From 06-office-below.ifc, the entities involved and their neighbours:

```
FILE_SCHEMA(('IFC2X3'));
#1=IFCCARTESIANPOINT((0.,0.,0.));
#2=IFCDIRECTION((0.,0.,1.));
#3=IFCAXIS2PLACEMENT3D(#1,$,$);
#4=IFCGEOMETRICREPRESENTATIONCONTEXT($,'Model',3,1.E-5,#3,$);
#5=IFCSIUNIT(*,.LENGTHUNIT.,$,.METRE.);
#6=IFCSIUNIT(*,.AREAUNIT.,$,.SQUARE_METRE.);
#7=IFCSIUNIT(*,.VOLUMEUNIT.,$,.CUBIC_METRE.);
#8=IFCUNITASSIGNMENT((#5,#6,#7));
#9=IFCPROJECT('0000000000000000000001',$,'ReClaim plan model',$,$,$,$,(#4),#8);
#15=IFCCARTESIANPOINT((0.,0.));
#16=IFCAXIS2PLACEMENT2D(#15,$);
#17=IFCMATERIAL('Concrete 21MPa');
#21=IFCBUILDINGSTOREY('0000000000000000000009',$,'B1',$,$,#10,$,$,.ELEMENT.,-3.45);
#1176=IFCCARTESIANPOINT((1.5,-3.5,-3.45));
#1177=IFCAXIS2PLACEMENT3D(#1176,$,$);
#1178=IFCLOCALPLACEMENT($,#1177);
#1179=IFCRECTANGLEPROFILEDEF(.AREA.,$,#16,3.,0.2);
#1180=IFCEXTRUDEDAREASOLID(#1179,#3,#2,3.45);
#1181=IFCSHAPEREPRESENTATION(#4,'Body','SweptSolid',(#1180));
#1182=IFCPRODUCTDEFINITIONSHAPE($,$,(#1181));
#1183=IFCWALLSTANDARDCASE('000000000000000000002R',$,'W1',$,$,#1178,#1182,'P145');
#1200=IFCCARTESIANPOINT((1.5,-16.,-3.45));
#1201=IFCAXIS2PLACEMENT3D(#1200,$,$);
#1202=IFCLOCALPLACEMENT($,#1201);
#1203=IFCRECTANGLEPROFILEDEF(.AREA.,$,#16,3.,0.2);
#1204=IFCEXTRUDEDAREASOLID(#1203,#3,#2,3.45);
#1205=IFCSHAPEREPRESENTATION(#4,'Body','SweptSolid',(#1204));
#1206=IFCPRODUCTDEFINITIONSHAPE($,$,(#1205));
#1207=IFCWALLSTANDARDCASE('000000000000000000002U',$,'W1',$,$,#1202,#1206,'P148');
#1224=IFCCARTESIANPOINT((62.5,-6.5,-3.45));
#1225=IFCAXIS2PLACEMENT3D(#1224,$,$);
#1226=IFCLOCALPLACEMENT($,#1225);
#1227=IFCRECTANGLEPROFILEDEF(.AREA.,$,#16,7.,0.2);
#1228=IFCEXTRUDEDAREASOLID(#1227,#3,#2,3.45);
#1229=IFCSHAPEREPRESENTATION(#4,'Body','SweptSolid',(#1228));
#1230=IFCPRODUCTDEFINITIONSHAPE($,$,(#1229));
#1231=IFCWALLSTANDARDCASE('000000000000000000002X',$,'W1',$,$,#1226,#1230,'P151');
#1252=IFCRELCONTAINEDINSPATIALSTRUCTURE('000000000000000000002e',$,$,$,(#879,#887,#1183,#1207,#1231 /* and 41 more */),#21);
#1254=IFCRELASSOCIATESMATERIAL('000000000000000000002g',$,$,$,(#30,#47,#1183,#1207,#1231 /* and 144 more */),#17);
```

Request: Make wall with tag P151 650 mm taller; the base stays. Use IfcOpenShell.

```python
import ifcopenshell
import ifcopenshell.geom
import ifcopenshell.util.shape
import ifcopenshell.util.unit

model = ifcopenshell.open("06-office-below.ifc")
unit_scale = ifcopenshell.util.unit.calculate_unit_scale(model)
settings = ifcopenshell.geom.settings()


def volume(element):
    """Net volume in cubic metres, openings subtracted."""
    shape = ifcopenshell.geom.create_shape(settings, element)
    return ifcopenshell.util.shape.get_volume(shape.geometry)


wall = model.by_guid("000000000000000000002X")
before = volume(wall)

body = next(r for r in wall.Representation.Representations if r.RepresentationIdentifier == "Body")
solid = body.Items[0]
old_height = solid.Depth
solid.Depth += 0.65 / unit_scale
after = volume(wall)

print(f"height {old_height:g} -> {solid.Depth:g}, volume {before:.3f} -> {after:.3f} m3")

model.write("06-office-below_edited.ifc")
```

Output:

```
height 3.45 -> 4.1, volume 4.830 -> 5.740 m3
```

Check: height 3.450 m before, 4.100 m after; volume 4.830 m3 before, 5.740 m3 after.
